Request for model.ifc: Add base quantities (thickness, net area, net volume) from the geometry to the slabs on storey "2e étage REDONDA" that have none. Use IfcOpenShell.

First a look at what the model holds.

```python
import ifcopenshell
import ifcopenshell.util.element
import ifcopenshell.util.unit

model = ifcopenshell.open("model.ifc")
print(model.schema)
for unit_type in ("LENGTHUNIT", "AREAUNIT", "VOLUMEUNIT"):
    print(unit_type, ifcopenshell.util.unit.calculate_unit_scale(model, unit_type))
storey = next(s for s in model.by_type("IfcBuildingStorey") if s.Name == "2e étage REDONDA")
slabs = [e for e in ifcopenshell.util.element.get_decomposition(storey) if e.is_a("IfcSlab")]
for e in sorted(slabs, key=lambda e: e.id()):
    print(e.id(), e.is_a(), e.Name, list(ifcopenshell.util.element.get_psets(e, qtos_only=True)), sep=" | ")
```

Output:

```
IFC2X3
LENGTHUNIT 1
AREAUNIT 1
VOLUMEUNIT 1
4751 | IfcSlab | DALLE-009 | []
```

```python
import ifcopenshell
import ifcopenshell.api.pset
import ifcopenshell.geom
import ifcopenshell.util.element
import ifcopenshell.util.shape
import ifcopenshell.util.unit

model = ifcopenshell.open("model.ifc")
unit_scale = ifcopenshell.util.unit.calculate_unit_scale(model)
area_scale = ifcopenshell.util.unit.calculate_unit_scale(model, "AREAUNIT")
volume_scale = ifcopenshell.util.unit.calculate_unit_scale(model, "VOLUMEUNIT")
settings = ifcopenshell.geom.settings()

storey = next(s for s in model.by_type("IfcBuildingStorey") if s.Name == "2e étage REDONDA")
slabs = [e for e in ifcopenshell.util.element.get_decomposition(storey) if e.is_a("IfcSlab")]

for e in sorted(slabs, key=lambda e: e.id()):
    if ifcopenshell.util.element.get_psets(e, qtos_only=True, should_inherit=False):
        continue
    # Geometry comes back in metres, in the element's own axes.
    shape = ifcopenshell.geom.create_shape(settings, e)
    values = {
        "Width": ifcopenshell.util.shape.get_z(shape.geometry) / unit_scale,
        "NetArea": ifcopenshell.util.shape.get_footprint_area(shape.geometry) / area_scale,
        "NetVolume": ifcopenshell.util.shape.get_volume(shape.geometry) / volume_scale,
    }
    qto = ifcopenshell.api.pset.add_qto(model, product=e, name="BaseQuantities")
    ifcopenshell.api.pset.edit_qto(model, qto=qto, properties=values)
    print(e.id(), {k: round(v, 3) for k, v in values.items()})

model.write("model_edited.ifc")
```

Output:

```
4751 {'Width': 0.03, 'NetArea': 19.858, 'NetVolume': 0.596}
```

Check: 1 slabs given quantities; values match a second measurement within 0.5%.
